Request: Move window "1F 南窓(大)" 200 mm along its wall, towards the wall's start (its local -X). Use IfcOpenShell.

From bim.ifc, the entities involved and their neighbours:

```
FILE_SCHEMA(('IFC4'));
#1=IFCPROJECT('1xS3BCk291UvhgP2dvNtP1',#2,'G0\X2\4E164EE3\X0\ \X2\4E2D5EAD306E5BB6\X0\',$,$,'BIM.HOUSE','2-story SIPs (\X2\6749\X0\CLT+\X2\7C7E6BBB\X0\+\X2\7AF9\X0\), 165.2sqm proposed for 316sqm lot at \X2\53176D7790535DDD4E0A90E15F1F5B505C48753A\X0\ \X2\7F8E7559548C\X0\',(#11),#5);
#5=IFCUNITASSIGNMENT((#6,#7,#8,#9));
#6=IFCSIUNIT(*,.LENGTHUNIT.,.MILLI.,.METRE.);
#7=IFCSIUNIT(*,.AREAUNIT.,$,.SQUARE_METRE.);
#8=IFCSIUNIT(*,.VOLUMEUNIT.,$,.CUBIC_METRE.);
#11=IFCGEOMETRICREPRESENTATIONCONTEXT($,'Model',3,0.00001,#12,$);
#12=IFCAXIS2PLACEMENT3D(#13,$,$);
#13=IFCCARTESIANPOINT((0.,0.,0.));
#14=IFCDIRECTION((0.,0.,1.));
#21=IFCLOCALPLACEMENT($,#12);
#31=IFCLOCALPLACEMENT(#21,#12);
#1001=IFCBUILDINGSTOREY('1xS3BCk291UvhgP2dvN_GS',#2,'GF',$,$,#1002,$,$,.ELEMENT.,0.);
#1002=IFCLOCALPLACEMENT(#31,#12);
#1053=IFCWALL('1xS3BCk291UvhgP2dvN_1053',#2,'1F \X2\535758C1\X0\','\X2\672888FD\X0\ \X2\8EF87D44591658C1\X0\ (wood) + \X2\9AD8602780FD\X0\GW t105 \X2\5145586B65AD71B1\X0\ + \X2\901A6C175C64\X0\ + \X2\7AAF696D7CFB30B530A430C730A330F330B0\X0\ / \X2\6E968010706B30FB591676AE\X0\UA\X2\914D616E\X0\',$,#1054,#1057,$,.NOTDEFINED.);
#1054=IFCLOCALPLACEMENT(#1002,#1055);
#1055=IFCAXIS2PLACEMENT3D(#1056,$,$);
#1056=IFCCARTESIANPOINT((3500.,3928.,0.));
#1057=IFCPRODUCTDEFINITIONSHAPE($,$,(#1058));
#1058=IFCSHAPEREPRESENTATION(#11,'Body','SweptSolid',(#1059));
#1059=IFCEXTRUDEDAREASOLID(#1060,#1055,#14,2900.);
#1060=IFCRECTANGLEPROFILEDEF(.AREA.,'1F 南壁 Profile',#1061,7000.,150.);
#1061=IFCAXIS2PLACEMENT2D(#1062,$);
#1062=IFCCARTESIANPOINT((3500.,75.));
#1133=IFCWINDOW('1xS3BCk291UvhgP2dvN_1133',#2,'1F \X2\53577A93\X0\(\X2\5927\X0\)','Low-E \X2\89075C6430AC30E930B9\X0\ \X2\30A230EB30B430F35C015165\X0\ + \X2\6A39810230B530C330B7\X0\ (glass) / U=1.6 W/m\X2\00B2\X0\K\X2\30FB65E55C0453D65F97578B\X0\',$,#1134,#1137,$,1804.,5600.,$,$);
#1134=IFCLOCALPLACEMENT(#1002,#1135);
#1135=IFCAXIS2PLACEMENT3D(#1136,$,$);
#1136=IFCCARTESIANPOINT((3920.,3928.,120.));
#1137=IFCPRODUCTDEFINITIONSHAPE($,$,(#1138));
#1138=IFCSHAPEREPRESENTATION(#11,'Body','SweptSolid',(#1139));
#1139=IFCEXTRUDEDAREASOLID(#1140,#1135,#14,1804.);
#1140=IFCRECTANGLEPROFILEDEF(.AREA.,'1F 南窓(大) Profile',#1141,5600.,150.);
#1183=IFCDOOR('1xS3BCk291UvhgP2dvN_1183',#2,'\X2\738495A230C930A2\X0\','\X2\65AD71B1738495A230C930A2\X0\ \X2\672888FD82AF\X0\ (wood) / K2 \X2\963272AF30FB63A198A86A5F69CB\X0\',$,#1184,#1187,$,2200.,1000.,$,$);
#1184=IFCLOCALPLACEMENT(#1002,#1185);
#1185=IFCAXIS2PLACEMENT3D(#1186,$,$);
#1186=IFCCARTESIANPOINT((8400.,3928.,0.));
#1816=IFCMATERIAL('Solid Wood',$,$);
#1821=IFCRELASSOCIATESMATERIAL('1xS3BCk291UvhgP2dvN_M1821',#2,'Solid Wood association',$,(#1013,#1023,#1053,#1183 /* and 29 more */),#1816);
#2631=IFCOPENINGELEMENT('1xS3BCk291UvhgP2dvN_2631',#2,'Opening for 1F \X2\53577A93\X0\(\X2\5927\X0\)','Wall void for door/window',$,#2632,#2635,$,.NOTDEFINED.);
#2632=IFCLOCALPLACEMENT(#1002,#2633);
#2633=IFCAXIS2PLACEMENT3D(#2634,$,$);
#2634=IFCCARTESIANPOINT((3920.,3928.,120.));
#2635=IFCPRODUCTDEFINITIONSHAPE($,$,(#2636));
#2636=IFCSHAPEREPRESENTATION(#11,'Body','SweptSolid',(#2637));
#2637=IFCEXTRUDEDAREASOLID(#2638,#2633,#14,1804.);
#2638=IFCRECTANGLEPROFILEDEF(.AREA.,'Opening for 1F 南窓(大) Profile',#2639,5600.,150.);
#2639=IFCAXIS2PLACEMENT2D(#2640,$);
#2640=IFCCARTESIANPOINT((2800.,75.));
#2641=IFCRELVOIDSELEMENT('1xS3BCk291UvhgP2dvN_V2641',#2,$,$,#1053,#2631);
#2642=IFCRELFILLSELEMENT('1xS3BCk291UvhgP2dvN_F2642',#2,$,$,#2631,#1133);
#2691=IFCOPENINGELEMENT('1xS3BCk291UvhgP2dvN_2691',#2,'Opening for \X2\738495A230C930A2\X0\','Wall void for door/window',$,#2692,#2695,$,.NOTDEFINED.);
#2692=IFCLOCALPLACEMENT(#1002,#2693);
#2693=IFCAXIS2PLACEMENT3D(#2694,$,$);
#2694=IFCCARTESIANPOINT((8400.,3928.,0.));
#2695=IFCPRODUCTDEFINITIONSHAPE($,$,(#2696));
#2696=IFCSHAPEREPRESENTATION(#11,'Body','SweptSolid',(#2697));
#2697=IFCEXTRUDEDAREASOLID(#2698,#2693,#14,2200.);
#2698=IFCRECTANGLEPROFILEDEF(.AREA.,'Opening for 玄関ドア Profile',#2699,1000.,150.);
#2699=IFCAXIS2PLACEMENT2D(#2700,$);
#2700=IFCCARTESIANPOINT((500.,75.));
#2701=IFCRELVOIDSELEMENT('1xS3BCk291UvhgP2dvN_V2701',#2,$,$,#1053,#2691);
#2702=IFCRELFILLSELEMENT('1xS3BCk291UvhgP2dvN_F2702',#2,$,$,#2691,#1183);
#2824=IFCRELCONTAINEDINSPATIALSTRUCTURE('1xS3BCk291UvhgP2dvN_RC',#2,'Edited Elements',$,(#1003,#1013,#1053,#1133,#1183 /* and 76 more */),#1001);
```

```python
import ifcopenshell
import ifcopenshell.api.geometry
import ifcopenshell.util.placement
import ifcopenshell.util.unit

model = ifcopenshell.open("bim.ifc")
unit_scale = ifcopenshell.util.unit.calculate_unit_scale(model)

window = model.by_guid("1xS3BCk291UvhgP2dvN_1133")
opening = window.FillsVoids[0].RelatingOpeningElement
wall = opening.VoidsElements[0].RelatingBuildingElement

wall_matrix = ifcopenshell.util.placement.get_local_placement(wall.ObjectPlacement)
shift = wall_matrix[:3, 0] * -0.2 / unit_scale
before = ifcopenshell.util.placement.get_local_placement(window.ObjectPlacement)[:3, 3].copy()

# The window is not placed relative to its opening, so move both.
for product in (opening, window):
    matrix = ifcopenshell.util.placement.get_local_placement(product.ObjectPlacement)
    matrix[:3, 3] += shift
    ifcopenshell.api.geometry.edit_object_placement(model, product=product, matrix=matrix, is_si=False)

after = ifcopenshell.util.placement.get_local_placement(window.ObjectPlacement)[:3, 3]
print("window moved by", (after - before).round(3) + 0.0)

model.write("bim_edited.ifc")
```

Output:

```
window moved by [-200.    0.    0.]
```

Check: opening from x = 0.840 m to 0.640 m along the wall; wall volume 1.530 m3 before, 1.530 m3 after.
